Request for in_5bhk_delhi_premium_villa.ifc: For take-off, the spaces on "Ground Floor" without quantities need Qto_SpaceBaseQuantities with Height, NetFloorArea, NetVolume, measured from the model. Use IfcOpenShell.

First a look at what the model holds.

```python
import ifcopenshell
import ifcopenshell.util.element
import ifcopenshell.util.unit

model = ifcopenshell.open("in_5bhk_delhi_premium_villa.ifc")
print(model.schema)
for unit_type in ("LENGTHUNIT", "AREAUNIT", "VOLUMEUNIT"):
    print(unit_type, ifcopenshell.util.unit.calculate_unit_scale(model, unit_type))
storey = next(s for s in model.by_type("IfcBuildingStorey") if s.Name == "Ground Floor")
spaces = [e for e in ifcopenshell.util.element.get_decomposition(storey) if e.is_a("IfcSpace")]
for e in sorted(spaces, key=lambda e: e.id()):
    print(e.id(), e.is_a(), e.Name, list(ifcopenshell.util.element.get_psets(e, qtos_only=True)), sep=" | ")
```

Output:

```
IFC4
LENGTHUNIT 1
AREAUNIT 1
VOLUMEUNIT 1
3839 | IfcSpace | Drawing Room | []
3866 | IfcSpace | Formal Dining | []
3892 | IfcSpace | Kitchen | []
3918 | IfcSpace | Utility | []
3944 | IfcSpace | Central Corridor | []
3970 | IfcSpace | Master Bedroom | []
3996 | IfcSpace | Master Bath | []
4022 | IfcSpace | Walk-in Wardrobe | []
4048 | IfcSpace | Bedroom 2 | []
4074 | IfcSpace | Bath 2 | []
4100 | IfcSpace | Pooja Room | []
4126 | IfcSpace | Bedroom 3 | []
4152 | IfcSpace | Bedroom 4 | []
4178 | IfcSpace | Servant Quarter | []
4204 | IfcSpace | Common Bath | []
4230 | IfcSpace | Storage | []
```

```python
import ifcopenshell
import ifcopenshell.api.pset
import ifcopenshell.geom
import ifcopenshell.util.element
import ifcopenshell.util.shape
import ifcopenshell.util.unit

model = ifcopenshell.open("in_5bhk_delhi_premium_villa.ifc")
unit_scale = ifcopenshell.util.unit.calculate_unit_scale(model)
area_scale = ifcopenshell.util.unit.calculate_unit_scale(model, "AREAUNIT")
volume_scale = ifcopenshell.util.unit.calculate_unit_scale(model, "VOLUMEUNIT")
settings = ifcopenshell.geom.settings()

storey = next(s for s in model.by_type("IfcBuildingStorey") if s.Name == "Ground Floor")
spaces = [e for e in ifcopenshell.util.element.get_decomposition(storey) if e.is_a("IfcSpace")]

for e in sorted(spaces, key=lambda e: e.id()):
    if ifcopenshell.util.element.get_psets(e, qtos_only=True, should_inherit=False):
        continue
    # Geometry comes back in metres, in the element's own axes.
    shape = ifcopenshell.geom.create_shape(settings, e)
    values = {
        "Height": ifcopenshell.util.shape.get_z(shape.geometry) / unit_scale,
        "NetFloorArea": ifcopenshell.util.shape.get_footprint_area(shape.geometry) / area_scale,
        "NetVolume": ifcopenshell.util.shape.get_volume(shape.geometry) / volume_scale,
    }
    qto = ifcopenshell.api.pset.add_qto(model, product=e, name="Qto_SpaceBaseQuantities")
    ifcopenshell.api.pset.edit_qto(model, qto=qto, properties=values)
    print(e.id(), {k: round(v, 3) for k, v in values.items()})

model.write("in_5bhk_delhi_premium_villa_edited.ifc")
```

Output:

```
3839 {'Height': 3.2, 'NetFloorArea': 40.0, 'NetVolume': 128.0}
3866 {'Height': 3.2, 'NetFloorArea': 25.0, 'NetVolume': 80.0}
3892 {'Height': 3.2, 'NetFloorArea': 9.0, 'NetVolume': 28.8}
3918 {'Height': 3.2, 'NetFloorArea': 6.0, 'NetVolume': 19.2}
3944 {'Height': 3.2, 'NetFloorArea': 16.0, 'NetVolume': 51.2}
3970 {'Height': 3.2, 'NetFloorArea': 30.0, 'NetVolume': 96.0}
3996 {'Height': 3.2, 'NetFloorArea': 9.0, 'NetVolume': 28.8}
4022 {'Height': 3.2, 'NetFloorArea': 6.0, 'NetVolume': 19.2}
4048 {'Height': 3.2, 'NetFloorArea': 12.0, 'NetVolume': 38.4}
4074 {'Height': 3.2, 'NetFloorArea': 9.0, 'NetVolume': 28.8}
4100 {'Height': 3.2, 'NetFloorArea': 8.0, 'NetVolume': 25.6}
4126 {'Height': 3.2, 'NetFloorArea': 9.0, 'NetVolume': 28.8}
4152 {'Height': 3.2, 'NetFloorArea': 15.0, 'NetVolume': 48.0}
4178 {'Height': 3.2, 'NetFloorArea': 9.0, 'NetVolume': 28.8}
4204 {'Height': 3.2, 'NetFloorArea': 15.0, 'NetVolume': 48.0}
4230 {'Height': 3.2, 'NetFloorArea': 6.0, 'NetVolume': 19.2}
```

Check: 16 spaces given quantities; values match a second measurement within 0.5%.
